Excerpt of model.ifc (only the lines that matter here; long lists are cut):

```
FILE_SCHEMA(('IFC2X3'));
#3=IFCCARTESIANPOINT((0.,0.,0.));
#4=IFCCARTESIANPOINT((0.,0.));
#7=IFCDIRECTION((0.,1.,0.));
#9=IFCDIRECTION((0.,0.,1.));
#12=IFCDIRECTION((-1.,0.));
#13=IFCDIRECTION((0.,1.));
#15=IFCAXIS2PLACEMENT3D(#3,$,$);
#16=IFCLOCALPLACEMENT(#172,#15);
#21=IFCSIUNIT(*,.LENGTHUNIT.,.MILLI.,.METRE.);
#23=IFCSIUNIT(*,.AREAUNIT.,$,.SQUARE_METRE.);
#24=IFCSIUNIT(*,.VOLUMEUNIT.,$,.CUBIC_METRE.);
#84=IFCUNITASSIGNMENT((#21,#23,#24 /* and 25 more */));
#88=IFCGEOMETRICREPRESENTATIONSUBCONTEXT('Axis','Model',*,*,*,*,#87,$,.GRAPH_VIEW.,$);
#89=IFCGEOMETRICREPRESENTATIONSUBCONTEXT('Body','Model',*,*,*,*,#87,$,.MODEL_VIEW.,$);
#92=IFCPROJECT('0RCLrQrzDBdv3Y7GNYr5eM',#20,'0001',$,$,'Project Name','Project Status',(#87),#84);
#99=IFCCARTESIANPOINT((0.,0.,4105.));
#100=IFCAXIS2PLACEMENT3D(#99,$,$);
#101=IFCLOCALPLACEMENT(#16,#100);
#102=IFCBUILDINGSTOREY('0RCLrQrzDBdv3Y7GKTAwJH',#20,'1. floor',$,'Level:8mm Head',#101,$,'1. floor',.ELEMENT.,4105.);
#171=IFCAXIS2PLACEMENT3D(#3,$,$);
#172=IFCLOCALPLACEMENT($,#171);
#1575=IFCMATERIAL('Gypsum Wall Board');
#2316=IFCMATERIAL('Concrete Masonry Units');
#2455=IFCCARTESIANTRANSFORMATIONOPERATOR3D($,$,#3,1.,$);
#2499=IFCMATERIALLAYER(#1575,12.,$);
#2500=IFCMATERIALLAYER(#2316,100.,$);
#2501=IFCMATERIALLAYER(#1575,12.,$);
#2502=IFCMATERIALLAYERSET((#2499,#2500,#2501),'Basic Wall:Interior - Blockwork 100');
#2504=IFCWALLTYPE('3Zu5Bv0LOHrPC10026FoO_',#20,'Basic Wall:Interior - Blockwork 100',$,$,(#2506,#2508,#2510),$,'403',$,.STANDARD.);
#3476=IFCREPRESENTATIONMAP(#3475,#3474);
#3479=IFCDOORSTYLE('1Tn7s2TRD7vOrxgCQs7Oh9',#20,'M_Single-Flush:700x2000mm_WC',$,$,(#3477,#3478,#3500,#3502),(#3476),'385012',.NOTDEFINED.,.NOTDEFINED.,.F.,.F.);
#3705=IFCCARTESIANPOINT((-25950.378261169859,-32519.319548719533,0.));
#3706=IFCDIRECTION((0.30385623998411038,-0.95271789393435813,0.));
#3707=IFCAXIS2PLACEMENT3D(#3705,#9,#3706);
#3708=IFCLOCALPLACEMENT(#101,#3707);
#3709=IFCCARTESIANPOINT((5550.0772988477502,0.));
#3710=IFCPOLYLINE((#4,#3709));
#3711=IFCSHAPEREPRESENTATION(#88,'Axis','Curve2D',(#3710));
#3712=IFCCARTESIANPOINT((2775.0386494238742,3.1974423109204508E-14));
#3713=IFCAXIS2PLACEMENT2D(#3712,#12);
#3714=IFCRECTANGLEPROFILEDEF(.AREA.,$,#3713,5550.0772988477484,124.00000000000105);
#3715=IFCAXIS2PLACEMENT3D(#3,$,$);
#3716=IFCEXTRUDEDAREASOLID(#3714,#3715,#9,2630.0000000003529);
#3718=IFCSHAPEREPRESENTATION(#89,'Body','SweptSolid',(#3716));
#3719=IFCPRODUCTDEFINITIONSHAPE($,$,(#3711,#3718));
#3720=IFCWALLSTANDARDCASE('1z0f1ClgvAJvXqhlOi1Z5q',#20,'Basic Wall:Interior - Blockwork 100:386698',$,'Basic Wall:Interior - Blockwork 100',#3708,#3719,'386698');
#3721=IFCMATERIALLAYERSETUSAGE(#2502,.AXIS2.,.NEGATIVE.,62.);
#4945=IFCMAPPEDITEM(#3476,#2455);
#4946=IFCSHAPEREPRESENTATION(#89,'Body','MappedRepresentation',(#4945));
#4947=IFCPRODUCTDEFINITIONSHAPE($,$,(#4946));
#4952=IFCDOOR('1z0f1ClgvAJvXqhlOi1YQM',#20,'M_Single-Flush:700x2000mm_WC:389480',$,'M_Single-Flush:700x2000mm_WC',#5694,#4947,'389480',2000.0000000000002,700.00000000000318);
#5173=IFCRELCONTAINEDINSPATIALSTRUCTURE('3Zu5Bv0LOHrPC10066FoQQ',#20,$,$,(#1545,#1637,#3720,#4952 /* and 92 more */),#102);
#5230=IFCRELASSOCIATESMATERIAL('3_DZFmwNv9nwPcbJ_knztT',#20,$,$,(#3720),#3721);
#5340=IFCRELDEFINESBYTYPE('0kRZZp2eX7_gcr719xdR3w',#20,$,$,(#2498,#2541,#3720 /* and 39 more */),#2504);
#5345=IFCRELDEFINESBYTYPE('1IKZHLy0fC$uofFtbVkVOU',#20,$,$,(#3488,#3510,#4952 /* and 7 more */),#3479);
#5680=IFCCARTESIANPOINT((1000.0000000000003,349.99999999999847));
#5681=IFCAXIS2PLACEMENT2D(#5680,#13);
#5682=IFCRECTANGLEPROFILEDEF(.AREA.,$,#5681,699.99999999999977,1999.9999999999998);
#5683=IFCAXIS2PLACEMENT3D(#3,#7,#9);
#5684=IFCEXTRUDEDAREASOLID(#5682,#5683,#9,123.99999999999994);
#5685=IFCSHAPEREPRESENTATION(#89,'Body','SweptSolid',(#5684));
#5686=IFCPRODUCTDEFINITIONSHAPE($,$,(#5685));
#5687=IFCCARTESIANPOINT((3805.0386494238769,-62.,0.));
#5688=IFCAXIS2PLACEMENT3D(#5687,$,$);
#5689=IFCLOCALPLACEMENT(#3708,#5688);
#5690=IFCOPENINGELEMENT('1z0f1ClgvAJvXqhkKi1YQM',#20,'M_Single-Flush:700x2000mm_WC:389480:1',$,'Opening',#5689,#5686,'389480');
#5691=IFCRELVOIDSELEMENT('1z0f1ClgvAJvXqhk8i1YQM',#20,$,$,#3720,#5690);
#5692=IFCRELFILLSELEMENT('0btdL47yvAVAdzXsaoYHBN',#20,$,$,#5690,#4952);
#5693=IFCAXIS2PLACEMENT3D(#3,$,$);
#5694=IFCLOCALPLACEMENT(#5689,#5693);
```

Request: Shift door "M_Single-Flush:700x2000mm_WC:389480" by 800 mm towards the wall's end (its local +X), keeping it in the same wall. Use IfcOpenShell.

```python
import ifcopenshell
import ifcopenshell.api.geometry
import ifcopenshell.util.placement

model = ifcopenshell.open("model.ifc")

door = model.by_id(4952)
opening = door.FillsVoids[0].RelatingOpeningElement
wall = opening.VoidsElements[0].RelatingBuildingElement

wall_matrix = ifcopenshell.util.placement.get_local_placement(wall.ObjectPlacement)
shift = wall_matrix[:3, 0] * 800.0
before = ifcopenshell.util.placement.get_local_placement(door.ObjectPlacement)[:3, 3].copy()

# The door is placed relative to its opening, so it follows when the opening moves.
matrix = ifcopenshell.util.placement.get_local_placement(opening.ObjectPlacement)
matrix[:3, 3] += shift
ifcopenshell.api.geometry.edit_object_placement(
    model, product=opening, matrix=matrix, is_si=False, should_transform_children=True
)

after = ifcopenshell.util.placement.get_local_placement(door.ObjectPlacement)[:3, 3]
print("door moved by", (after - before).round(3) + 0.0)

model.write("model_v2.ifc")
```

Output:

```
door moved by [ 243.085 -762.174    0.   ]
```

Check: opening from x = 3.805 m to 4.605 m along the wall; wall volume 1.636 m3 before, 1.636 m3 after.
